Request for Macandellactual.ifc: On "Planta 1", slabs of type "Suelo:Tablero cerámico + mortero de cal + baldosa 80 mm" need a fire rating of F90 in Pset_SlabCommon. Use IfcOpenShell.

First a look at what the model holds.

```python
import ifcopenshell
import ifcopenshell.util.element

model = ifcopenshell.open("Macandellactual.ifc")
print(model.schema)
storey = next(s for s in model.by_type("IfcBuildingStorey") if s.Name == "Planta 1")
slabs = [e for e in ifcopenshell.util.element.get_decomposition(storey) if e.is_a("IfcSlab")]
seen = {}
for e in slabs:
    element_type = ifcopenshell.util.element.get_type(e)
    key = (element_type.Name if element_type != e and element_type else None, ifcopenshell.util.element.get_pset(e, "Pset_SlabCommon", "FireRating"))
    seen[key] = seen.get(key, 0) + 1
for (name, value), count in sorted(seen.items(), key=str):
    print(count, "x", name, "|", value)
```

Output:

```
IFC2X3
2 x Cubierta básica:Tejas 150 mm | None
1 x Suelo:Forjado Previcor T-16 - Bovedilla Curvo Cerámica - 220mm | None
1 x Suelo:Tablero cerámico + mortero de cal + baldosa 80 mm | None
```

```python
import ifcopenshell
import ifcopenshell.api.pset
import ifcopenshell.util.element

model = ifcopenshell.open("Macandellactual.ifc")

storey = next(s for s in model.by_type("IfcBuildingStorey") if s.Name == "Planta 1")
slabs = [e for e in ifcopenshell.util.element.get_decomposition(storey) if e.is_a("IfcSlab")]

count = 0
for e in slabs:
    element_type = ifcopenshell.util.element.get_type(e)
    if element_type in (None, e) or element_type.Name != "Suelo:Tablero cerámico + mortero de cal + baldosa 80 mm":
        continue
    # add_pset returns the element's existing set when there is one.
    pset = ifcopenshell.api.pset.add_pset(model, product=e, name="Pset_SlabCommon")
    ifcopenshell.api.pset.edit_pset(model, pset=pset, properties={"FireRating": "F90"})
    count += 1

print(count, "slabs updated")

model.write("Macandellactual_rev.ifc")
```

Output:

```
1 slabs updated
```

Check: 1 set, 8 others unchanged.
